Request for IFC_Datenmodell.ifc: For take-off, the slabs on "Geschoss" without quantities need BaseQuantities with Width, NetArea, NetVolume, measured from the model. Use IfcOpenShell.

First a look at what the model holds.

```python
import ifcopenshell
import ifcopenshell.util.element
import ifcopenshell.util.unit

model = ifcopenshell.open("IFC_Datenmodell.ifc")
print(model.schema)
for unit_type in ("LENGTHUNIT", "AREAUNIT", "VOLUMEUNIT"):
    print(unit_type, ifcopenshell.util.unit.calculate_unit_scale(model, unit_type))
storey = next(s for s in model.by_type("IfcBuildingStorey") if s.Name == "Geschoss")
slabs = [e for e in ifcopenshell.util.element.get_decomposition(storey) if e.is_a("IfcSlab")]
for e in sorted(slabs, key=lambda e: e.id()):
    print(e.id(), e.is_a(), e.Name, list(ifcopenshell.util.element.get_psets(e, qtos_only=True)), sep=" | ")
```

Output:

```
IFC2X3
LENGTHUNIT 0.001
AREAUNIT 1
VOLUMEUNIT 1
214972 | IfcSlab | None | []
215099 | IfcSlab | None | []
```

```python
import ifcopenshell
import ifcopenshell.api.pset
import ifcopenshell.geom
import ifcopenshell.util.element
import ifcopenshell.util.shape
import ifcopenshell.util.unit

model = ifcopenshell.open("IFC_Datenmodell.ifc")
unit_scale = ifcopenshell.util.unit.calculate_unit_scale(model)
area_scale = ifcopenshell.util.unit.calculate_unit_scale(model, "AREAUNIT")
volume_scale = ifcopenshell.util.unit.calculate_unit_scale(model, "VOLUMEUNIT")
settings = ifcopenshell.geom.settings()

storey = next(s for s in model.by_type("IfcBuildingStorey") if s.Name == "Geschoss")
slabs = [e for e in ifcopenshell.util.element.get_decomposition(storey) if e.is_a("IfcSlab")]

for e in sorted(slabs, key=lambda e: e.id()):
    if ifcopenshell.util.element.get_psets(e, qtos_only=True, should_inherit=False):
        continue
    # Geometry comes back in metres, in the element's own axes.
    shape = ifcopenshell.geom.create_shape(settings, e)
    values = {
        "Width": ifcopenshell.util.shape.get_z(shape.geometry) / unit_scale,
        "NetArea": ifcopenshell.util.shape.get_footprint_area(shape.geometry) / area_scale,
        "NetVolume": ifcopenshell.util.shape.get_volume(shape.geometry) / volume_scale,
    }
    qto = ifcopenshell.api.pset.add_qto(model, product=e, name="BaseQuantities")
    ifcopenshell.api.pset.edit_qto(model, qto=qto, properties=values)
    print(e.id(), {k: round(v, 3) for k, v in values.items()})

model.write("IFC_Datenmodell_updated.ifc")
```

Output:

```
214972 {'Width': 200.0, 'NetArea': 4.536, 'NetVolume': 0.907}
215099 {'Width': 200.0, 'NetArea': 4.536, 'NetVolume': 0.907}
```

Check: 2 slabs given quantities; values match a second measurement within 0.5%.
